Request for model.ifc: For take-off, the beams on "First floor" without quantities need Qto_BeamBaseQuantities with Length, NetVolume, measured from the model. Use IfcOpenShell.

First a look at what the model holds.

```python
import ifcopenshell
import ifcopenshell.util.element
import ifcopenshell.util.unit

model = ifcopenshell.open("model.ifc")
print(model.schema)
for unit_type in ("LENGTHUNIT", "AREAUNIT", "VOLUMEUNIT"):
    print(unit_type, ifcopenshell.util.unit.calculate_unit_scale(model, unit_type))
storey = next(s for s in model.by_type("IfcBuildingStorey") if s.Name == "First floor")
beams = [e for e in ifcopenshell.util.element.get_decomposition(storey) if e.is_a("IfcBeam")]
for e in sorted(beams, key=lambda e: e.id()):
    print(e.id(), e.is_a(), e.Name, list(ifcopenshell.util.element.get_psets(e, qtos_only=True)), sep=" | ")
```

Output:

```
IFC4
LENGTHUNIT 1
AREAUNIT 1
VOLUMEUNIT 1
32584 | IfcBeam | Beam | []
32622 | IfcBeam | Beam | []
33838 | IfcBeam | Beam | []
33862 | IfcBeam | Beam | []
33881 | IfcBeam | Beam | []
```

```python
import ifcopenshell
import ifcopenshell.api.pset
import ifcopenshell.geom
import ifcopenshell.util.element
import ifcopenshell.util.shape
import ifcopenshell.util.unit

model = ifcopenshell.open("model.ifc")
unit_scale = ifcopenshell.util.unit.calculate_unit_scale(model)
volume_scale = ifcopenshell.util.unit.calculate_unit_scale(model, "VOLUMEUNIT")
settings = ifcopenshell.geom.settings()

storey = next(s for s in model.by_type("IfcBuildingStorey") if s.Name == "First floor")
beams = [e for e in ifcopenshell.util.element.get_decomposition(storey) if e.is_a("IfcBeam")]

for e in sorted(beams, key=lambda e: e.id()):
    if ifcopenshell.util.element.get_psets(e, qtos_only=True, should_inherit=False):
        continue
    # Geometry comes back in metres, in the element's own axes.
    shape = ifcopenshell.geom.create_shape(settings, e)
    values = {
        "Length": ifcopenshell.util.shape.get_max_xyz(shape.geometry) / unit_scale,
        "NetVolume": ifcopenshell.util.shape.get_volume(shape.geometry) / volume_scale,
    }
    qto = ifcopenshell.api.pset.add_qto(model, product=e, name="Qto_BeamBaseQuantities")
    ifcopenshell.api.pset.edit_qto(model, qto=qto, properties=values)
    print(e.id(), {k: round(v, 3) for k, v in values.items()})

model.write("model-out.ifc")
```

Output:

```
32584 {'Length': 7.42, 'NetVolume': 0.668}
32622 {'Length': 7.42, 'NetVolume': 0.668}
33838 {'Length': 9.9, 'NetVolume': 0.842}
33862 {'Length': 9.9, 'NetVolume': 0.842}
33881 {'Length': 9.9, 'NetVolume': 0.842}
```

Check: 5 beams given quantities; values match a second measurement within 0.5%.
